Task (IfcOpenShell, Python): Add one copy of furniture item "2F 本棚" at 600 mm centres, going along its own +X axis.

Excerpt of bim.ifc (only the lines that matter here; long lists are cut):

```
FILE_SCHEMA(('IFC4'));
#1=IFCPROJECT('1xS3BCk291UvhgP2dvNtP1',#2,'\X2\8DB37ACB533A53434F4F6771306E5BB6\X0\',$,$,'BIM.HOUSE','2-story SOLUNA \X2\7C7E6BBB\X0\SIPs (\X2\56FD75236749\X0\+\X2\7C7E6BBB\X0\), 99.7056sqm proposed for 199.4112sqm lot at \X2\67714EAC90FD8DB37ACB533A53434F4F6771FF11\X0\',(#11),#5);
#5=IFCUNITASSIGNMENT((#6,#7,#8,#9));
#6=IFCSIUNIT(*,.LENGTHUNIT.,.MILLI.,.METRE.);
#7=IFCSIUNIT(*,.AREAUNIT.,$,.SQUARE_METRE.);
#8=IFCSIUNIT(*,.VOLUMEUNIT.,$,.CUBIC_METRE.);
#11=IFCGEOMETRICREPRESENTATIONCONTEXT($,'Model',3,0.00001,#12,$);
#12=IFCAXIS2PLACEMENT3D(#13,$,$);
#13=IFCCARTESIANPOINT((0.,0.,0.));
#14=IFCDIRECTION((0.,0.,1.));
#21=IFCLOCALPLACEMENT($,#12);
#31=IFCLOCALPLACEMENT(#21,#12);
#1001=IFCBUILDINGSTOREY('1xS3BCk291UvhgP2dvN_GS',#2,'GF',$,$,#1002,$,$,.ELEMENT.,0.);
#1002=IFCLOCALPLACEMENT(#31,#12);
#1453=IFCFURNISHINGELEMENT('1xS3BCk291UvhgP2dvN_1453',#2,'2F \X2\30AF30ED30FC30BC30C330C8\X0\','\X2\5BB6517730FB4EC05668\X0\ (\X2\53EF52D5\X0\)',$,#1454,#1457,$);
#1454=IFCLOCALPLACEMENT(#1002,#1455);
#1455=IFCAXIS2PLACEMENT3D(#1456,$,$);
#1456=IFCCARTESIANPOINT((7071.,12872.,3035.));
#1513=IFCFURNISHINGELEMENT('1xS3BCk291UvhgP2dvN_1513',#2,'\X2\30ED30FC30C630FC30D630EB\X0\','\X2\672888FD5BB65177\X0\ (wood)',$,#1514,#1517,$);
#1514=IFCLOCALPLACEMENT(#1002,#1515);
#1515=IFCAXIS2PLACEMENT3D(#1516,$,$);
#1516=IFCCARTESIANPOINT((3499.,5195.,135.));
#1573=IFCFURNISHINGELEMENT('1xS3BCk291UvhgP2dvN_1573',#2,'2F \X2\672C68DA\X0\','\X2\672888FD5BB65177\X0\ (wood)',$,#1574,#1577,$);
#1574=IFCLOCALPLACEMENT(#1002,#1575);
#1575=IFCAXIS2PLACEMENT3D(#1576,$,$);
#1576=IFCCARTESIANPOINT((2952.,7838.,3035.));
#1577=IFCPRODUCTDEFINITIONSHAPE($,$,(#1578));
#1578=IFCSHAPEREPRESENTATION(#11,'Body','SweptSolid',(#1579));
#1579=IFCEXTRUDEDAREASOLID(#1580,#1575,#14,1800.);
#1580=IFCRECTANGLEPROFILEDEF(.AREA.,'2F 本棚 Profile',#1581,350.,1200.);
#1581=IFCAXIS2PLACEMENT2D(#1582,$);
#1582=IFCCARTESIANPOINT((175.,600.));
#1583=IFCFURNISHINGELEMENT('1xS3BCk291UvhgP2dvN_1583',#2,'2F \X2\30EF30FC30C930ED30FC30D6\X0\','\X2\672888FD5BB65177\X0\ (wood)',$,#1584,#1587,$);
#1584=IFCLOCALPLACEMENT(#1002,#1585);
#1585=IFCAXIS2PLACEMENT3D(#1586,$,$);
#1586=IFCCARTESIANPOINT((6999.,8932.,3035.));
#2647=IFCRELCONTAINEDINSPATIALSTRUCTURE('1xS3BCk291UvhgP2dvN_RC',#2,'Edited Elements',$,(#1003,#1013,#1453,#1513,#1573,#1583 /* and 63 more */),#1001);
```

```python
import ifcopenshell
import ifcopenshell.api.geometry
import ifcopenshell.api.root
import ifcopenshell.util.element
import ifcopenshell.util.placement
import ifcopenshell.util.unit

model = ifcopenshell.open("bim.ifc")
unit_scale = ifcopenshell.util.unit.calculate_unit_scale(model)


def reuse_history(source, copy):
    """copy_class also copies each property set's owner history, people and application; keep the originals."""
    for rel in copy.IsDefinedBy:
        if rel.is_a("IfcRelDefinesByProperties") and (history := rel.RelatingPropertyDefinition.OwnerHistory):
            rel.RelatingPropertyDefinition.OwnerHistory = source.OwnerHistory
            ifcopenshell.util.element.remove_deep2(model, history)


source = model.by_guid("1xS3BCk291UvhgP2dvN_1573")
base = ifcopenshell.util.placement.get_local_placement(source.ObjectPlacement)
step = base[:3, 0] * 0.6 / unit_scale

for i in range(1, 2):
    copy = ifcopenshell.api.root.copy_class(model, product=source)
    copy.Representation = ifcopenshell.util.element.copy_deep(
        model, source.Representation, exclude=["IfcGeometricRepresentationContext", "IfcRepresentationMap"]
    )
    reuse_history(source, copy)
    matrix = base.copy()
    matrix[:3, 3] += i * step
    print("added at", matrix[:3, 3].round(3) + 0.0)
    ifcopenshell.api.geometry.edit_object_placement(model, product=copy, matrix=matrix, is_si=False)

model.write("bim-out.ifc")
```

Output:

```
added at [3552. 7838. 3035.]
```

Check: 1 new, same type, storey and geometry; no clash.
